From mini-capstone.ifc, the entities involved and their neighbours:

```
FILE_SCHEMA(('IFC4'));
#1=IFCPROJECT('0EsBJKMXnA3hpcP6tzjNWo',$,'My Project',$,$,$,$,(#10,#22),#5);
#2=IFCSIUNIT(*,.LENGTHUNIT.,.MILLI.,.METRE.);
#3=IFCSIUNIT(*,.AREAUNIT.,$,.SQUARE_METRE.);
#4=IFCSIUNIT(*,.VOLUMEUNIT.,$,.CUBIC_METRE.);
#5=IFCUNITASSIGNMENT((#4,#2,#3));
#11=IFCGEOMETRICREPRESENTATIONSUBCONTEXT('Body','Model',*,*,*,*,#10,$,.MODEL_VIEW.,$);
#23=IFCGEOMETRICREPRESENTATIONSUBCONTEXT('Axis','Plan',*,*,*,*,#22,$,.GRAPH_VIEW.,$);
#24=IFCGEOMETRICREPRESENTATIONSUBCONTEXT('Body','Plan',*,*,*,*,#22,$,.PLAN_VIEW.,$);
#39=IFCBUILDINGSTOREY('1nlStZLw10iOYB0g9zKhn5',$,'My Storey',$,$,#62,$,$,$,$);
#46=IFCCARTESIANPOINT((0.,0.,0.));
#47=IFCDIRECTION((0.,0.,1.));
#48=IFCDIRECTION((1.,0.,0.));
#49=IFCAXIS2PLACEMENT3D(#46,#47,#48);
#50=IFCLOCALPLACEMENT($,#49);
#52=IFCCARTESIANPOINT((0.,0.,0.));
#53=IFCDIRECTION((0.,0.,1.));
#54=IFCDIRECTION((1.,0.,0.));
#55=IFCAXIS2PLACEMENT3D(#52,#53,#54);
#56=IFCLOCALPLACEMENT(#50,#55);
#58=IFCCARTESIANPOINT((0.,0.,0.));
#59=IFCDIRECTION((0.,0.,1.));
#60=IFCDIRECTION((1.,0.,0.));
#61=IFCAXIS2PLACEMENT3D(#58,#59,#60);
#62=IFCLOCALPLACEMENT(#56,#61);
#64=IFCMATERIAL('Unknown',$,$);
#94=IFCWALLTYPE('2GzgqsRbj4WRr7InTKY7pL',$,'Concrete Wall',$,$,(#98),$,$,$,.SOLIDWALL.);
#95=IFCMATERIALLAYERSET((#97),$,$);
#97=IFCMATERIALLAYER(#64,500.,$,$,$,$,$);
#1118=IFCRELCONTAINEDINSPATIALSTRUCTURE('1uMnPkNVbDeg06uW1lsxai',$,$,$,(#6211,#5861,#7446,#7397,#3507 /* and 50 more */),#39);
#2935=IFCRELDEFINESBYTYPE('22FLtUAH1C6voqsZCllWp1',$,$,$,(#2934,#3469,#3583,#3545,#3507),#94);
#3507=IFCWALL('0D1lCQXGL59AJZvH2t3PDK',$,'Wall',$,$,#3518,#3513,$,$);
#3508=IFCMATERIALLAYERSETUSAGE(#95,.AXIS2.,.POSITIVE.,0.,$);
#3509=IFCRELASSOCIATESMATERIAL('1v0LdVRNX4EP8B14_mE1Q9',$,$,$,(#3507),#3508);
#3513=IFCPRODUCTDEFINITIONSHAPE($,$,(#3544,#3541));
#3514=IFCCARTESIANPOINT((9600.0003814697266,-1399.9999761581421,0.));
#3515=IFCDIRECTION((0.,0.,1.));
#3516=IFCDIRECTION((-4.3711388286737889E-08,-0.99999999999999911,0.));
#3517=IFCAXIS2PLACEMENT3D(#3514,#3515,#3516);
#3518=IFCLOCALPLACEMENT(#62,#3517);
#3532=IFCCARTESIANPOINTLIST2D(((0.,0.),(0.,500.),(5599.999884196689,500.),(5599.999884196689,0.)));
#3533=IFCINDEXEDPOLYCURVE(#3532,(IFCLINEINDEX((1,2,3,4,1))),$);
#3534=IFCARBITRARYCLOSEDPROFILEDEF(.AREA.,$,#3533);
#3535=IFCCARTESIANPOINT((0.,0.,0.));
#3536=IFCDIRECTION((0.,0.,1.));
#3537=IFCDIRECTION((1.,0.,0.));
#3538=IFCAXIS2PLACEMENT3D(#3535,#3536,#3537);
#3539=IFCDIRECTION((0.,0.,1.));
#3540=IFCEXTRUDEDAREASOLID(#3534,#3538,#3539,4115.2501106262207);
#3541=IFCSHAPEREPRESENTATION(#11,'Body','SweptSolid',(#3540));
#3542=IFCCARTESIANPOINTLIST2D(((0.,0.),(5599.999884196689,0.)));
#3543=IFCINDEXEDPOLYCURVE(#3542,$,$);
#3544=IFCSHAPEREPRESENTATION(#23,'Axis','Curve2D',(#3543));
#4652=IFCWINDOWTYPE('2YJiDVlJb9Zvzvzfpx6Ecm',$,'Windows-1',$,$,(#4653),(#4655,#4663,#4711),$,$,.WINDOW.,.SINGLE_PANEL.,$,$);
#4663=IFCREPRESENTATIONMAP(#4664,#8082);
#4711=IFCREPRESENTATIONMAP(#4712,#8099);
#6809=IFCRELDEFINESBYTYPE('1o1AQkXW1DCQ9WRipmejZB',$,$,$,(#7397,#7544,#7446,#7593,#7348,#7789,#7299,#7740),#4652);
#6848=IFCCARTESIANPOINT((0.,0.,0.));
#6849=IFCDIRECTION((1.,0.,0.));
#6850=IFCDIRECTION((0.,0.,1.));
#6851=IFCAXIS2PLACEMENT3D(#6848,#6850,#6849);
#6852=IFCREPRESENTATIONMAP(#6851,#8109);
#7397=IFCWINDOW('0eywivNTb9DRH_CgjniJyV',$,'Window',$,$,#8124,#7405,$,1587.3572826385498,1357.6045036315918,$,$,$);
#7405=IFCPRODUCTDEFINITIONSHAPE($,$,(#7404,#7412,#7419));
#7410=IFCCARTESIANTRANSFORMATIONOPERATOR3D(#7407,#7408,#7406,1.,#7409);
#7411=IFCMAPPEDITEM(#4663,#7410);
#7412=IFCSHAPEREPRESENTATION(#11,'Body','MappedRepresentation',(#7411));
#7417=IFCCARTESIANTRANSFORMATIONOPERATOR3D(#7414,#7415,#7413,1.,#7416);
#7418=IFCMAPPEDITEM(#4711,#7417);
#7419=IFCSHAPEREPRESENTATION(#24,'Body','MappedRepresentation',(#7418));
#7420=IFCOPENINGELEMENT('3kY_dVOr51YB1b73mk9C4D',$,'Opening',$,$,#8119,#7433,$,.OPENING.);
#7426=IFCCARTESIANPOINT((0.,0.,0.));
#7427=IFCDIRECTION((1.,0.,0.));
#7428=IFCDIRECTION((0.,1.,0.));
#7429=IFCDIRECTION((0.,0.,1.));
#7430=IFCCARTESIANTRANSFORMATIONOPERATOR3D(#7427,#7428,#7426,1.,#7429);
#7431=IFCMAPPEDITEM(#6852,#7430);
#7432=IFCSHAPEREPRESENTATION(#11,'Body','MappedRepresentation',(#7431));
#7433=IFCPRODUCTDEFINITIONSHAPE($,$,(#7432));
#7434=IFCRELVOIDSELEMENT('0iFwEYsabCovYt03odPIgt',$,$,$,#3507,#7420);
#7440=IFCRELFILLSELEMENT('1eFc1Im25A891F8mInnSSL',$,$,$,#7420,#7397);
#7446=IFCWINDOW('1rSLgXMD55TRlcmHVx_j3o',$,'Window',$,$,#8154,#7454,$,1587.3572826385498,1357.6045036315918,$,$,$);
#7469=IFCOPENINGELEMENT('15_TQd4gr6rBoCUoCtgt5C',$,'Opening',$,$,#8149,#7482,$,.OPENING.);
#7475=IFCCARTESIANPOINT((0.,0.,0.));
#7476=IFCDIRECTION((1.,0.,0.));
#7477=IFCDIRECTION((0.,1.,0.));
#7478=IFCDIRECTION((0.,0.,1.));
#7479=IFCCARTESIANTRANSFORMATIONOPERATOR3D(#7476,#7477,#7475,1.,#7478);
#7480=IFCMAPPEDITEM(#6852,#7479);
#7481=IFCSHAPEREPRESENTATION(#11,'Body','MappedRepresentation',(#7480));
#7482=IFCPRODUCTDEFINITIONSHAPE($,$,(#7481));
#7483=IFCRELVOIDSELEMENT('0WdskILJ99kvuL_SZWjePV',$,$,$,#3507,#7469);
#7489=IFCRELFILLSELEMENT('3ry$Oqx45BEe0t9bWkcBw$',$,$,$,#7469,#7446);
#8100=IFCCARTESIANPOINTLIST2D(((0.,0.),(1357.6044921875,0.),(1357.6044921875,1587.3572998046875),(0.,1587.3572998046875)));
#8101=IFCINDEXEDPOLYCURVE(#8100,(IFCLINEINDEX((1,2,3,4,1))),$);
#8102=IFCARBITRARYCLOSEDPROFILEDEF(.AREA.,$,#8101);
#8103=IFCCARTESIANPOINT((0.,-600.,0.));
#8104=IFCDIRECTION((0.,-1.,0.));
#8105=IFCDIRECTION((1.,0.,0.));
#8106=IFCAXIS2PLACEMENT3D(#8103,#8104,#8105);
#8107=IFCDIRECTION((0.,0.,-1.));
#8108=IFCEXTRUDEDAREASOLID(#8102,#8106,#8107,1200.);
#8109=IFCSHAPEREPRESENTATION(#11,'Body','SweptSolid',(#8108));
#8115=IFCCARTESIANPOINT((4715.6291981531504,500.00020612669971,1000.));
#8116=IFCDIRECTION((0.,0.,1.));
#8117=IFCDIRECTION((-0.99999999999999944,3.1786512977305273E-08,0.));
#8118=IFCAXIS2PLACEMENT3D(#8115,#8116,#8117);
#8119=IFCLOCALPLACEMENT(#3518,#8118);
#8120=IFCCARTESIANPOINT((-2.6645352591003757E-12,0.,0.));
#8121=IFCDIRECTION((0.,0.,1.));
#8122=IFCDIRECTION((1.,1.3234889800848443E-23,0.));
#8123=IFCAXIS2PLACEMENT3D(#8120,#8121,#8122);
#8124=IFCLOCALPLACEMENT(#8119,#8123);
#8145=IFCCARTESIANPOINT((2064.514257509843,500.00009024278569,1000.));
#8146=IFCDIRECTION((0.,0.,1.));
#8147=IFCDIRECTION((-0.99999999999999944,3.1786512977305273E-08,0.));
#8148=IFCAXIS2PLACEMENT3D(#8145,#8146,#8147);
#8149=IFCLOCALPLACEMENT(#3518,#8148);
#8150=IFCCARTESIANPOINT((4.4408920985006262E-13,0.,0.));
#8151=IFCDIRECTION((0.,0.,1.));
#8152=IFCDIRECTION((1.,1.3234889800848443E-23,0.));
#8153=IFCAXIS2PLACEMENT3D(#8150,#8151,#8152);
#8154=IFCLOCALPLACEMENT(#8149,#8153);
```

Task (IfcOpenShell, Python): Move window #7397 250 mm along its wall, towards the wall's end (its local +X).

```python
import ifcopenshell
import ifcopenshell.api.geometry
import ifcopenshell.util.placement
import ifcopenshell.util.unit

model = ifcopenshell.open("mini-capstone.ifc")
unit_scale = ifcopenshell.util.unit.calculate_unit_scale(model)

window = model.by_id(7397)
opening = window.FillsVoids[0].RelatingOpeningElement
wall = opening.VoidsElements[0].RelatingBuildingElement

wall_matrix = ifcopenshell.util.placement.get_local_placement(wall.ObjectPlacement)
shift = wall_matrix[:3, 0] * 0.25 / unit_scale
before = ifcopenshell.util.placement.get_local_placement(window.ObjectPlacement)[:3, 3].copy()

# The window is placed relative to its opening, so it follows when the opening moves.
matrix = ifcopenshell.util.placement.get_local_placement(opening.ObjectPlacement)
matrix[:3, 3] += shift
ifcopenshell.api.geometry.edit_object_placement(
    model, product=opening, matrix=matrix, is_si=False, should_transform_children=True
)

after = ifcopenshell.util.placement.get_local_placement(window.ObjectPlacement)[:3, 3]
print("window moved by", (after - before).round(3) + 0.0)

model.write("mini-capstone-out.ifc")
```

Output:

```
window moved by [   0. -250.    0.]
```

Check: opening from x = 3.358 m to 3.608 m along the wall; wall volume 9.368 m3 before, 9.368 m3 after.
